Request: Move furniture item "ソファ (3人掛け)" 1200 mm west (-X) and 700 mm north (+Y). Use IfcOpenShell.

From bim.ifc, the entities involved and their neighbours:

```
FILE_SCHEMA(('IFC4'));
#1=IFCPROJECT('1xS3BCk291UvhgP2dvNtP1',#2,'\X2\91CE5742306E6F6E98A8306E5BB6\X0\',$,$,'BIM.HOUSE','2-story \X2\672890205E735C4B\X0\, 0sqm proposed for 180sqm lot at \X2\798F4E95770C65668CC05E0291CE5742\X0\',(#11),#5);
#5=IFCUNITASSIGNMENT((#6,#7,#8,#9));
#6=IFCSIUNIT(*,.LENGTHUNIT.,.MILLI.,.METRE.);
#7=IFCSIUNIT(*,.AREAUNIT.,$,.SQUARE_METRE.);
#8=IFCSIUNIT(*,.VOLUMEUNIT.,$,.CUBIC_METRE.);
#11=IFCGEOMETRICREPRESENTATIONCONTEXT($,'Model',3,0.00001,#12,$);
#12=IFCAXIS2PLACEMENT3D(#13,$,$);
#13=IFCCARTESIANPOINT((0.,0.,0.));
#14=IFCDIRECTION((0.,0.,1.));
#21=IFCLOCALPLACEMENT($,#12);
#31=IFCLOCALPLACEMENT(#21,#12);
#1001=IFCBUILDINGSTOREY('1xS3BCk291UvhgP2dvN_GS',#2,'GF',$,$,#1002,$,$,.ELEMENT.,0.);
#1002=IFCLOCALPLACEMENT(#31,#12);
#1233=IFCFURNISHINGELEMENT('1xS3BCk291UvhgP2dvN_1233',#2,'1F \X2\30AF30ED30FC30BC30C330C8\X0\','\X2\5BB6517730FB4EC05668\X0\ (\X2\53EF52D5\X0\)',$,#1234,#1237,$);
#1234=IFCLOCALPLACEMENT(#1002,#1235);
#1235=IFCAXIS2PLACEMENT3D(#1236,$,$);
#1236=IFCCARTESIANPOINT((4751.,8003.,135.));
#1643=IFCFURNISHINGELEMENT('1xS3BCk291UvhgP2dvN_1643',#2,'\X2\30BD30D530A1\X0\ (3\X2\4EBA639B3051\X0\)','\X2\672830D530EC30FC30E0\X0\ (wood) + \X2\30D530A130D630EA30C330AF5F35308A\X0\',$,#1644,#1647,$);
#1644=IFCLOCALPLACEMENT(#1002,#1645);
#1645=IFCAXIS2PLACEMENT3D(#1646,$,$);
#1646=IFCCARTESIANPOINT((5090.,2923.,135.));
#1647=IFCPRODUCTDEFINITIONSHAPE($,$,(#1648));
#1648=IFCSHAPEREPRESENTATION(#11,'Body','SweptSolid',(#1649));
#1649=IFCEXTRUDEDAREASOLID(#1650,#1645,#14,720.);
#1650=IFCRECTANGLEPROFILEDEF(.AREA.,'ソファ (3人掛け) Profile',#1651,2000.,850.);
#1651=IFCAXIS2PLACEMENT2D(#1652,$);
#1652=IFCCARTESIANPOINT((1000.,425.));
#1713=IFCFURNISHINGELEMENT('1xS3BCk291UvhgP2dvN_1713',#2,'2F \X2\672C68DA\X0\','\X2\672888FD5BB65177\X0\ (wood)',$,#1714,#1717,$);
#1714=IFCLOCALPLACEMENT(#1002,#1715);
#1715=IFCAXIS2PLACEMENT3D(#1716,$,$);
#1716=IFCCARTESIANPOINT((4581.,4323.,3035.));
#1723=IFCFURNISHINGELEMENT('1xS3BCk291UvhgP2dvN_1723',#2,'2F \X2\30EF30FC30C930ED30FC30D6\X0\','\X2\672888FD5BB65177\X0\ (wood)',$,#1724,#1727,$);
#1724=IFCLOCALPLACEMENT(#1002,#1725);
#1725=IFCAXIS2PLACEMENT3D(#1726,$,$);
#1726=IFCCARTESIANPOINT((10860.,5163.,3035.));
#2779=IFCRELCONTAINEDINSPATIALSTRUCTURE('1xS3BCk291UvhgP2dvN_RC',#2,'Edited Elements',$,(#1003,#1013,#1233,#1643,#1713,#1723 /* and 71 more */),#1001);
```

```python
import ifcopenshell
import ifcopenshell.api.geometry
import ifcopenshell.util.placement

model = ifcopenshell.open("bim.ifc")

item = model.by_guid("1xS3BCk291UvhgP2dvN_1643")
matrix = ifcopenshell.util.placement.get_local_placement(item.ObjectPlacement)
matrix[0, 3] -= 1200.0
matrix[1, 3] += 700.0
ifcopenshell.api.geometry.edit_object_placement(model, product=item, matrix=matrix, is_si=False)

print(ifcopenshell.util.placement.get_local_placement(item.ObjectPlacement).round(3) + 0.0)

model.write("bim_updated.ifc")
```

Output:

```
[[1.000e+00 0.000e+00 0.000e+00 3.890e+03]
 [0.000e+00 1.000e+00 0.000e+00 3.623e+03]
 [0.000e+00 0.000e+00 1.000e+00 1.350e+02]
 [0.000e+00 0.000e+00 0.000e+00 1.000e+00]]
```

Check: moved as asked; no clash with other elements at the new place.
